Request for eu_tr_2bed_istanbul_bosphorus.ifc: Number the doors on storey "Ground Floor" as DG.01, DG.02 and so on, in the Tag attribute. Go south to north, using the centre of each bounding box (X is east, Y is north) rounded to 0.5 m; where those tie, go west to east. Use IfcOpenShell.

First a look at what the model holds.

```python
import ifcopenshell
import ifcopenshell.util.element
import ifcopenshell.util.placement

model = ifcopenshell.open("eu_tr_2bed_istanbul_bosphorus.ifc")
print(model.schema)
storey = next(s for s in model.by_type("IfcBuildingStorey") if s.Name == "Ground Floor")
doors = [e for e in ifcopenshell.util.element.get_decomposition(storey) if e.is_a("IfcDoor")]
for e in sorted(doors, key=lambda e: e.id()):
    origin = ifcopenshell.util.placement.get_local_placement(e.ObjectPlacement)[:3, 3]
    print(e.id(), e.Tag, e.Name, origin.round(2) + 0.0, sep=" | ")
```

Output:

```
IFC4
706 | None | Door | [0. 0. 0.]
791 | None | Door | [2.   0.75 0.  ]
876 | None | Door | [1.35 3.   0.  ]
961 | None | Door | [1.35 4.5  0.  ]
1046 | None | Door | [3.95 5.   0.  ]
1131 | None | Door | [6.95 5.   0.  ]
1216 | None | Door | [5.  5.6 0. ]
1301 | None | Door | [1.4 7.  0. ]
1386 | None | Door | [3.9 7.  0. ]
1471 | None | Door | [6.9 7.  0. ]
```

```python
import ifcopenshell
import ifcopenshell.geom
import ifcopenshell.util.element
import ifcopenshell.util.shape

model = ifcopenshell.open("eu_tr_2bed_istanbul_bosphorus.ifc")
settings = ifcopenshell.geom.settings()
settings.set("use-world-coords", True)


def centre(element):
    shape = ifcopenshell.geom.create_shape(settings, element)
    return ifcopenshell.util.shape.get_bbox_centroid(shape.geometry)


storey = next(s for s in model.by_type("IfcBuildingStorey") if s.Name == "Ground Floor")
doors = [e for e in ifcopenshell.util.element.get_decomposition(storey) if e.is_a("IfcDoor")]

# Insertion points can sit at a corner or the storey origin, so sort by the geometry (in metres).
centres = {e: centre(e) for e in doors}
doors.sort(key=lambda e: (round(centres[e][1] / 0.5), centres[e][0]))

for i, e in enumerate(doors, start=1):
    number = f"DG.{i:02d}"
    e.Tag = number
    print(e.id(), number)

model.write("eu_tr_2bed_istanbul_bosphorus_v2.ifc")
```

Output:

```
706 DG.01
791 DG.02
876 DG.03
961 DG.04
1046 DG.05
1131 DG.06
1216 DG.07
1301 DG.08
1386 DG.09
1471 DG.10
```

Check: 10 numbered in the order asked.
